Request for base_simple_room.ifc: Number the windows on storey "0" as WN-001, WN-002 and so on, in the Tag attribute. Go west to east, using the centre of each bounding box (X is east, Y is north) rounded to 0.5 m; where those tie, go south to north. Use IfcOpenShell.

First a look at what the model holds.

```python
import ifcopenshell
import ifcopenshell.util.element
import ifcopenshell.util.placement

model = ifcopenshell.open("base_simple_room.ifc")
print(model.schema)
storey = next(s for s in model.by_type("IfcBuildingStorey") if s.Name == "0")
windows = [e for e in ifcopenshell.util.element.get_decomposition(storey) if e.is_a("IfcWindow")]
for e in sorted(windows, key=lambda e: e.id()):
    origin = ifcopenshell.util.placement.get_local_placement(e.ObjectPlacement)[:3, 3]
    print(e.id(), e.Tag, e.Name, origin.round(2) + 0.0, sep=" | ")
```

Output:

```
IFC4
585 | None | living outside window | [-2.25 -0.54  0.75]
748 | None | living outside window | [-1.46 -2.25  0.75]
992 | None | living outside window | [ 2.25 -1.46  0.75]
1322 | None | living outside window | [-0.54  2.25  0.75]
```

```python
import ifcopenshell
import ifcopenshell.geom
import ifcopenshell.util.element
import ifcopenshell.util.shape

model = ifcopenshell.open("base_simple_room.ifc")
settings = ifcopenshell.geom.settings()
settings.set("use-world-coords", True)


def centre(element):
    shape = ifcopenshell.geom.create_shape(settings, element)
    return ifcopenshell.util.shape.get_bbox_centroid(shape.geometry)


storey = next(s for s in model.by_type("IfcBuildingStorey") if s.Name == "0")
windows = [e for e in ifcopenshell.util.element.get_decomposition(storey) if e.is_a("IfcWindow")]

# Insertion points can sit at a corner or the storey origin, so sort by the geometry (in metres).
centres = {e: centre(e) for e in windows}
windows.sort(key=lambda e: (round(centres[e][0] / 0.5), centres[e][1]))

for i, e in enumerate(windows, start=1):
    number = f"WN-0{i:02d}"
    e.Tag = number
    print(e.id(), number)

model.write("base_simple_room_v2.ifc")
```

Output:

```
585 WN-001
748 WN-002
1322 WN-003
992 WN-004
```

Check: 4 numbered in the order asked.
